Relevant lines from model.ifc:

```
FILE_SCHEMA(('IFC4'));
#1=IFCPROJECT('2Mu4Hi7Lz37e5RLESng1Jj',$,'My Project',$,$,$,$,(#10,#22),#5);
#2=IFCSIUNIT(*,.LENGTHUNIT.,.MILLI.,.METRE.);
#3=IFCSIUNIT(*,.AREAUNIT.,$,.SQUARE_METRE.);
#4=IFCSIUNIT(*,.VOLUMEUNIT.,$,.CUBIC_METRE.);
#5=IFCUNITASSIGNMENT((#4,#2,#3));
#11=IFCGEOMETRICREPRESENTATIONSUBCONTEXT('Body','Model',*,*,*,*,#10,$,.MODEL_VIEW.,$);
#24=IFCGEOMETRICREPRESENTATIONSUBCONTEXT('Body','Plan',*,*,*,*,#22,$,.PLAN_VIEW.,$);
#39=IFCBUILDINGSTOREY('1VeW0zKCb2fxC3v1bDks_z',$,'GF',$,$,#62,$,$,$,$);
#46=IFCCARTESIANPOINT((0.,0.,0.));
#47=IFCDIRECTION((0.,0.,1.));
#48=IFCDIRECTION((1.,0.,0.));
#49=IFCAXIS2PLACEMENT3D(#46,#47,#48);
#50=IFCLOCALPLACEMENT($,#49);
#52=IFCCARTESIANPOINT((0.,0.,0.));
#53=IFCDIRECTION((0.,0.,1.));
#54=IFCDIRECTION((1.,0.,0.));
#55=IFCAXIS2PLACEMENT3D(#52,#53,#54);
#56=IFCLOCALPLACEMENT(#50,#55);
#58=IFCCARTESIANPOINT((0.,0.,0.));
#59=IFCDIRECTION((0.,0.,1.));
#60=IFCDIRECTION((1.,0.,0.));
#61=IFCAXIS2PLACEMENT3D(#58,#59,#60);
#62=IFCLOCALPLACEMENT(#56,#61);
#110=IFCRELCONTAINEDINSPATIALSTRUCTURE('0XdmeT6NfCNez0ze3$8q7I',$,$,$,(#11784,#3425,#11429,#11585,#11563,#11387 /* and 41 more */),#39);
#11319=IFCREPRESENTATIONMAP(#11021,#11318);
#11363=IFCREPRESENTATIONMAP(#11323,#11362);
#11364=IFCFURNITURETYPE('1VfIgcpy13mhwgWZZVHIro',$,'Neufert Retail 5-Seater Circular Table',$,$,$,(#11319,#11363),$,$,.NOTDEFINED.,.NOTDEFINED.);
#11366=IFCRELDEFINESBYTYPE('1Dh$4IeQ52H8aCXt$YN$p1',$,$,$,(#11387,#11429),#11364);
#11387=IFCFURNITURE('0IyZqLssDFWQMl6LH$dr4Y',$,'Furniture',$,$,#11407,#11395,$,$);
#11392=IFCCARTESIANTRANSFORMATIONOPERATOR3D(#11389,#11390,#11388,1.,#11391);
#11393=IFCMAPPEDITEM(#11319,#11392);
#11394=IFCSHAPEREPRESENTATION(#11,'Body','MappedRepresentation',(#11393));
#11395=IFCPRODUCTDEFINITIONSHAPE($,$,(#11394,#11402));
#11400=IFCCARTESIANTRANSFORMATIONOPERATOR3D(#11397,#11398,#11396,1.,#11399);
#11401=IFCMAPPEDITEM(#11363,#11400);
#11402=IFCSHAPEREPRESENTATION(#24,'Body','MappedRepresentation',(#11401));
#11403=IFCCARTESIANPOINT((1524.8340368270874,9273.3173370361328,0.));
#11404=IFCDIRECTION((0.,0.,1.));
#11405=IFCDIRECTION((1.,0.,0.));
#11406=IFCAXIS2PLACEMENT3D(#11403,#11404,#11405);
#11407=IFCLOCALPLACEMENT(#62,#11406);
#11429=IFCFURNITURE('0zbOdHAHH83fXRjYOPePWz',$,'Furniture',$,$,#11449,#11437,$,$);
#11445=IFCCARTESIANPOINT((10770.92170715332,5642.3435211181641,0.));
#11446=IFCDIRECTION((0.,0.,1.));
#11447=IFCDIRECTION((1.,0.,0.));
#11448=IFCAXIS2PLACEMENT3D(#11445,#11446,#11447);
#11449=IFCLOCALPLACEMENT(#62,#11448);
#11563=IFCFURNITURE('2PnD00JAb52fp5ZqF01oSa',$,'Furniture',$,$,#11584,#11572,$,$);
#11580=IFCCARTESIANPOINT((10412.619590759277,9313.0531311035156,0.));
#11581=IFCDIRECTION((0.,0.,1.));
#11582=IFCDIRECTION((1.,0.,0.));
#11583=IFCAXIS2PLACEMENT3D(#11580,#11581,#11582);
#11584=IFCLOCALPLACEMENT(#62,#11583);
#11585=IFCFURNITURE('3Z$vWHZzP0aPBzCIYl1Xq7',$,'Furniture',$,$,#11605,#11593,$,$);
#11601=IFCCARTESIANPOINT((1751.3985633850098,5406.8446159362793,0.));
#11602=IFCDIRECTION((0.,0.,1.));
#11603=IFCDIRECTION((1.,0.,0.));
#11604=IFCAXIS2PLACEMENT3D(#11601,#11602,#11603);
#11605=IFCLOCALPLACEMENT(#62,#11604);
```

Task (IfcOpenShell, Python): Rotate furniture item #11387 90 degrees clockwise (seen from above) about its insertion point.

```python
import ifcopenshell
import ifcopenshell.api.geometry
import ifcopenshell.util.placement

model = ifcopenshell.open("model.ifc")

item = model.by_guid("0IyZqLssDFWQMl6LH$dr4Y")
matrix = ifcopenshell.util.placement.get_local_placement(item.ObjectPlacement)
matrix = matrix @ ifcopenshell.util.placement.rotation(-90, "Z")
ifcopenshell.api.geometry.edit_object_placement(model, product=item, matrix=matrix, is_si=False)

print(ifcopenshell.util.placement.get_local_placement(item.ObjectPlacement).round(3) + 0.0)

model.write("model_edited.ifc")
```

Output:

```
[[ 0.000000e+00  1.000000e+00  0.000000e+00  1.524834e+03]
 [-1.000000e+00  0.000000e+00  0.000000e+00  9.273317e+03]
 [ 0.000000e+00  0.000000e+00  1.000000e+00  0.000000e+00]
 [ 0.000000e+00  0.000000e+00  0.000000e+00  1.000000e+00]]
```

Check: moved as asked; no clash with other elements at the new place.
